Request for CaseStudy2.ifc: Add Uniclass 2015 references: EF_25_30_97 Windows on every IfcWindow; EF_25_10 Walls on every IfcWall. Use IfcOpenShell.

First a look at what the model holds.

```python
import ifcopenshell

model = ifcopenshell.open("CaseStudy2.ifc")
print(model.schema)
print("classifications:", [c.Name for c in model.by_type("IfcClassification")])
for ifc_class in ("IfcDoor", "IfcRoof", "IfcStair", "IfcWall", "IfcWindow"):
    print(ifc_class, len(model.by_type(ifc_class)))
```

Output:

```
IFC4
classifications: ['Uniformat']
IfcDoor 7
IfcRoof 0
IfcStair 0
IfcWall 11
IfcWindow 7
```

```python
import ifcopenshell
import ifcopenshell.api.classification

model = ifcopenshell.open("CaseStudy2.ifc")

system = ifcopenshell.api.classification.add_classification(model, classification="Uniclass 2015")

codes = {
    "IfcWindow": ("EF_25_30_97", "Windows"),
    "IfcWall": ("EF_25_10", "Walls"),
}
for ifc_class, (code, name) in codes.items():
    products = model.by_type(ifc_class)
    ifcopenshell.api.classification.add_reference(
        model, products=products, classification=system, identification=code, name=name
    )
    print(code, len(products))

model.write("CaseStudy2_updated.ifc")
```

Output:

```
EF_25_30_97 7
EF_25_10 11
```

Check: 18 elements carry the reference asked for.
